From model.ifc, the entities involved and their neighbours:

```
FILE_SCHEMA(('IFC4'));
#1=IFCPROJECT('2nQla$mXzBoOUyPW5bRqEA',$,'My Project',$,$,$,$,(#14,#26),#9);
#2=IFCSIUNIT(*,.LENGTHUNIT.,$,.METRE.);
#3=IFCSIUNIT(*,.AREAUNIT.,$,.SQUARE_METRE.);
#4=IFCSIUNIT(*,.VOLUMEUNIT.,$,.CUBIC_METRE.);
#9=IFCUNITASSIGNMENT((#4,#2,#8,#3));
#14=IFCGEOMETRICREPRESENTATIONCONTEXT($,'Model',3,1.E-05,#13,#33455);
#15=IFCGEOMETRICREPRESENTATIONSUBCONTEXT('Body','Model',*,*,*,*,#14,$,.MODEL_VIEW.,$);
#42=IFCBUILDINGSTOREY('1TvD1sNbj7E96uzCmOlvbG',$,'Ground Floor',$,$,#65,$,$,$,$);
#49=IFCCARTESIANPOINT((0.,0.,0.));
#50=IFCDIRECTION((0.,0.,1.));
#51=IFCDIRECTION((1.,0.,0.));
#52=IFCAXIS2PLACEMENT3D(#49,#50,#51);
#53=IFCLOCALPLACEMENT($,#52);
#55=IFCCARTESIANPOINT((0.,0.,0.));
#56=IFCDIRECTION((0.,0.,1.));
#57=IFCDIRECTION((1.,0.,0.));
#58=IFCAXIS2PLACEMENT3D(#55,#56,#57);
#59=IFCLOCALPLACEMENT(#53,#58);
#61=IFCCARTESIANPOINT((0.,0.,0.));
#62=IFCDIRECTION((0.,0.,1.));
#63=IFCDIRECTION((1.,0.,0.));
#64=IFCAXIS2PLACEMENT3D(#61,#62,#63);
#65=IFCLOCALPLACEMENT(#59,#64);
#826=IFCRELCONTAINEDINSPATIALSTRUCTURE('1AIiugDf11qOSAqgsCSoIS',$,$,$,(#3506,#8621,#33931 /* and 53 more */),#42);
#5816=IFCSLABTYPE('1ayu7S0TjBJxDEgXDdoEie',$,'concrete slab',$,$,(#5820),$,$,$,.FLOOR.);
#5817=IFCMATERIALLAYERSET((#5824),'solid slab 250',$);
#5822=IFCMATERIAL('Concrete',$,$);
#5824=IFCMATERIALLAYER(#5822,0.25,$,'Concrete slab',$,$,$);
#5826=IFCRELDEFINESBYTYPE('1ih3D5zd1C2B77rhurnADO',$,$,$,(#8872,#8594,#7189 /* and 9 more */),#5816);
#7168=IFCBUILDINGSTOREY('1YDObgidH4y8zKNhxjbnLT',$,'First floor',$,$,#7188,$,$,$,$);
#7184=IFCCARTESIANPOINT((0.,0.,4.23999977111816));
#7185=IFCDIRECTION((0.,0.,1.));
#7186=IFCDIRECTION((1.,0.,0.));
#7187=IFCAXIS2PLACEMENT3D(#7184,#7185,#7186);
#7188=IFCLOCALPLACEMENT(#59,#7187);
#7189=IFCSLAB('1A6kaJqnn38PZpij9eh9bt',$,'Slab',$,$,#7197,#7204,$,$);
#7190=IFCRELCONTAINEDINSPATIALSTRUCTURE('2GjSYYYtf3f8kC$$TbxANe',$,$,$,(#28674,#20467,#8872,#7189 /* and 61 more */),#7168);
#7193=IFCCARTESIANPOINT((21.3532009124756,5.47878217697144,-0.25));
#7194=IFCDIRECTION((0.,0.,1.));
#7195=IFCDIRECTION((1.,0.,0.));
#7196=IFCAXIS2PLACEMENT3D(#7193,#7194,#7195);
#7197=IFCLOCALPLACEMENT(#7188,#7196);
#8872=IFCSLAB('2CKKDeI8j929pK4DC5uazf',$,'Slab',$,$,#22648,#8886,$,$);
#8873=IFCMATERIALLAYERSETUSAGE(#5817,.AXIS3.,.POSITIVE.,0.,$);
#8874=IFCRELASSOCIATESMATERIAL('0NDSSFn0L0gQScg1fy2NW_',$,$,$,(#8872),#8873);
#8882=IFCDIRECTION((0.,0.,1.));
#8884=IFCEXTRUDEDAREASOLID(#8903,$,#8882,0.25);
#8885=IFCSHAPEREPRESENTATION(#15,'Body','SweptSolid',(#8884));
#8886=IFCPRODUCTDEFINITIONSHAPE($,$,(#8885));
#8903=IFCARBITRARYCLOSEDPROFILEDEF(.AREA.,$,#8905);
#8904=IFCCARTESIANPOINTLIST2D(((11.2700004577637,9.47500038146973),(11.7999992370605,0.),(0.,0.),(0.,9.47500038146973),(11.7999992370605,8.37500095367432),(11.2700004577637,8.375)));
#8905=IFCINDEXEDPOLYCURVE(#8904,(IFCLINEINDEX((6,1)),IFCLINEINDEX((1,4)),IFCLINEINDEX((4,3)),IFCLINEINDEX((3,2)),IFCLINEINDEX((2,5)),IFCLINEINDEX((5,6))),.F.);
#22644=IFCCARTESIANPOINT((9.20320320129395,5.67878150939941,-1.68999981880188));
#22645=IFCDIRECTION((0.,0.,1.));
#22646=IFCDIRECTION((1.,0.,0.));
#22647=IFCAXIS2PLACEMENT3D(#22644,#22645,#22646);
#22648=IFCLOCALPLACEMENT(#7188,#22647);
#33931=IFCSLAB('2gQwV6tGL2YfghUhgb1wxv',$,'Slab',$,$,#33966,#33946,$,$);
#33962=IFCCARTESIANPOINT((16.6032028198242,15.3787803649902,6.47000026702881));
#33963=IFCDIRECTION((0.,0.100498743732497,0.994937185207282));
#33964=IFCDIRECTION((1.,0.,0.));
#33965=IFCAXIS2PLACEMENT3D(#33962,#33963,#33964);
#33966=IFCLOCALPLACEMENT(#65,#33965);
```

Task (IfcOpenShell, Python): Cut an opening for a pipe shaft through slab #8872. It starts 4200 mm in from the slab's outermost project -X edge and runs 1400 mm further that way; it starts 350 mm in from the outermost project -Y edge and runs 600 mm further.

```python
import numpy as np
import ifcopenshell
import ifcopenshell.api.feature
import ifcopenshell.api.geometry
import ifcopenshell.api.root
import ifcopenshell.geom
import ifcopenshell.util.placement
import ifcopenshell.util.representation
import ifcopenshell.util.shape
import ifcopenshell.util.unit

model = ifcopenshell.open("model.ifc")
unit_scale = ifcopenshell.util.unit.calculate_unit_scale(model)
settings = ifcopenshell.geom.settings()


def volume(element):
    """Net volume in cubic metres, openings subtracted."""
    shape = ifcopenshell.geom.create_shape(settings, element)
    return ifcopenshell.util.shape.get_volume(shape.geometry)


slab = model.by_id(8872)
before = volume(slab)

# Extent in the slab's own axes, in metres. The edges named are its -X and -Y sides.
slab_shape = ifcopenshell.geom.create_shape(settings, slab)
vertices = ifcopenshell.util.shape.get_vertices(slab_shape.geometry)
x_min, y_min, bottom = vertices.min(axis=0)
top = vertices[:, 2].max()

opening = ifcopenshell.api.root.create_entity(model, ifc_class="IfcOpeningElement", name="Pipe shaft opening", predefined_type="OPENING")
context = ifcopenshell.util.representation.get_context(model, "Model", "Body", "MODEL_VIEW")
width, depth = 1.4, 0.6
outline = [(0.0, 0.0), (width, 0.0), (width, depth), (0.0, depth), (0.0, 0.0)]
# Overshoot both faces by 50 mm so the cut is clean.
shape = ifcopenshell.api.geometry.add_slab_representation(
    model, context=context, depth=top - bottom + 0.1, polyline=outline
)
ifcopenshell.api.geometry.assign_representation(model, product=opening, representation=shape)

matrix = ifcopenshell.util.placement.get_local_placement(slab.ObjectPlacement)
matrix[:, 3] = matrix @ np.append(np.array([x_min + 4.2, y_min + 0.35, bottom - 0.05]) / unit_scale, 1.0)
ifcopenshell.api.geometry.edit_object_placement(model, product=opening, matrix=matrix, is_si=False)
ifcopenshell.api.feature.add_feature(model, feature=opening, element=slab)

after = volume(slab)

print(f"slab volume {before:.3f} -> {after:.3f} m3")

model.write("model_v2.ifc")
```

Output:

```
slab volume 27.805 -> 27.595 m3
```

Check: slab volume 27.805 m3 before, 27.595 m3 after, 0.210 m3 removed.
